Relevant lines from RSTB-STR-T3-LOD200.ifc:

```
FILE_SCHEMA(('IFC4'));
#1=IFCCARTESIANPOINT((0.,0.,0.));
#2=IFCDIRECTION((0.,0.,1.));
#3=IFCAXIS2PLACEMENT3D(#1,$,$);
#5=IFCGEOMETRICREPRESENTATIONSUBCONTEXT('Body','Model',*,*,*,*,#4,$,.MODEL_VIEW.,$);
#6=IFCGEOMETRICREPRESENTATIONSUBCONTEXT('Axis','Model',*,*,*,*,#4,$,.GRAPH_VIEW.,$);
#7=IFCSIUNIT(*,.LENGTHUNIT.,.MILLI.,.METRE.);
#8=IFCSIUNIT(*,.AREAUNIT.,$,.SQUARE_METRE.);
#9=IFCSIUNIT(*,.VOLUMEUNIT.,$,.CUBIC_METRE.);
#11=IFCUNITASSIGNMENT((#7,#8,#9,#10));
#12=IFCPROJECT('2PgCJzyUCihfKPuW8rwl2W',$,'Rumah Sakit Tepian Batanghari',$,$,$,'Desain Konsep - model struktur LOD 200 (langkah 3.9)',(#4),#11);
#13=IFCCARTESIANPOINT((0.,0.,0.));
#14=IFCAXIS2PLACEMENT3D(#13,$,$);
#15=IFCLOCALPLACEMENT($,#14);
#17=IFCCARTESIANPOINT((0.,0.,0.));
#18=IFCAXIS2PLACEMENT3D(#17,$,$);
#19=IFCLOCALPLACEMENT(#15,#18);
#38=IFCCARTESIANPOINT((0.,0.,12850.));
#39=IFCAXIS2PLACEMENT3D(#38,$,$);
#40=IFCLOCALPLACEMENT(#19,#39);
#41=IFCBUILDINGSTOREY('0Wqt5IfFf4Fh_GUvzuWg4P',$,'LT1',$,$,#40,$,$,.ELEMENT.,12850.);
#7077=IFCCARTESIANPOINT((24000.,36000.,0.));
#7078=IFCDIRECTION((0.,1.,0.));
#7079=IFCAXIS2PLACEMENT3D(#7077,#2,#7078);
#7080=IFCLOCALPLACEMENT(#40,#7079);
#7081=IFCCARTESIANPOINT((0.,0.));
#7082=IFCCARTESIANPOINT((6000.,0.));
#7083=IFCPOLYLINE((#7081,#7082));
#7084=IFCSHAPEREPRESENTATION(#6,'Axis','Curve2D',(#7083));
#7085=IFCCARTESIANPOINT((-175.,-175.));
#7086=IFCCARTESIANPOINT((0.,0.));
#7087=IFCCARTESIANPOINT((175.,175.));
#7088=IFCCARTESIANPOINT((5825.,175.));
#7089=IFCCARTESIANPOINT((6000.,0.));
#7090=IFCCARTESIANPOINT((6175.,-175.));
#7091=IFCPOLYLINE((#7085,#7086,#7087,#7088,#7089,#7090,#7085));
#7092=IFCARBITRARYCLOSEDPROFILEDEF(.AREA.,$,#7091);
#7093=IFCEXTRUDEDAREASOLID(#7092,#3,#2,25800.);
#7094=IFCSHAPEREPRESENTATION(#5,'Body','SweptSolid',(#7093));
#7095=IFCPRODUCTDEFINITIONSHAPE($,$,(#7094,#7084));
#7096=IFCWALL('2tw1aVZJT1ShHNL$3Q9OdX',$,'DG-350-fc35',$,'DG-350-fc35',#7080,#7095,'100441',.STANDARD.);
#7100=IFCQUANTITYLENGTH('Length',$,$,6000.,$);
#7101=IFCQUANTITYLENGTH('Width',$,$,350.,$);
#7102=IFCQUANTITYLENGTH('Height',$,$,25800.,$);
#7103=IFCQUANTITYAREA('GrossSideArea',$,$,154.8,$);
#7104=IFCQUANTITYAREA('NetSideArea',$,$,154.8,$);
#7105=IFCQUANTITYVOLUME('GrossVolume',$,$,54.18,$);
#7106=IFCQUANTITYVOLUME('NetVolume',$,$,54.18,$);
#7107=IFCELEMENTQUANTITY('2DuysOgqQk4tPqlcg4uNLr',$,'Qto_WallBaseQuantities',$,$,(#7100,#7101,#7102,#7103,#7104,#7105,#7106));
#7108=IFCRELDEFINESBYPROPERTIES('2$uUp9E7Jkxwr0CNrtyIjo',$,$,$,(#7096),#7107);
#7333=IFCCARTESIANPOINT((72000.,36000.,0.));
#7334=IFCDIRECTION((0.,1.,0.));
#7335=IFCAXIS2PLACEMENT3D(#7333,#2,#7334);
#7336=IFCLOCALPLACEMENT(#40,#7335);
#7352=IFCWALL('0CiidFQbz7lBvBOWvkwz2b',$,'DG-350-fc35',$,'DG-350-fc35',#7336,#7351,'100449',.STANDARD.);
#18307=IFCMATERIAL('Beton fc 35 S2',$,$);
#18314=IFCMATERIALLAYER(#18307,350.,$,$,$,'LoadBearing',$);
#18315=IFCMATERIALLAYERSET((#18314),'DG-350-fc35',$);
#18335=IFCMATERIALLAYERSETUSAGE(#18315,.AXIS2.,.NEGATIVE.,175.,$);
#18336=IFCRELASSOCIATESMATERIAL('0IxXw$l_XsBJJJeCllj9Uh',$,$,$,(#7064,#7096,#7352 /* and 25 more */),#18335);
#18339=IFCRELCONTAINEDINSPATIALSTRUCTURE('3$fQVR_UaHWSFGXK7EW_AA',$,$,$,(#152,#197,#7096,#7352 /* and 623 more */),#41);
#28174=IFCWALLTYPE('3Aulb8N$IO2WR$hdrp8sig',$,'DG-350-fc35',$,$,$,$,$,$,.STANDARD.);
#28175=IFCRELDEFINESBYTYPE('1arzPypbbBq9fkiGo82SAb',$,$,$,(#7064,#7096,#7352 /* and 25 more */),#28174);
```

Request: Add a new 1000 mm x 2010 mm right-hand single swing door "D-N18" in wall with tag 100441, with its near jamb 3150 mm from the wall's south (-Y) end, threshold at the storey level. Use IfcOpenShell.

```python
import numpy as np
import ifcopenshell
import ifcopenshell.api.feature
import ifcopenshell.api.geometry
import ifcopenshell.api.pset
import ifcopenshell.api.root
import ifcopenshell.api.spatial
import ifcopenshell.geom
import ifcopenshell.util.element
import ifcopenshell.util.placement
import ifcopenshell.util.representation
import ifcopenshell.util.shape
import ifcopenshell.util.unit

model = ifcopenshell.open("RSTB-STR-T3-LOD200.ifc")
unit_scale = ifcopenshell.util.unit.calculate_unit_scale(model)
area_scale = ifcopenshell.util.unit.calculate_unit_scale(model, "AREAUNIT")
volume_scale = ifcopenshell.util.unit.calculate_unit_scale(model, "VOLUMEUNIT")
settings = ifcopenshell.geom.settings()


def volume(element):
    """Net volume in cubic metres, openings subtracted."""
    shape = ifcopenshell.geom.create_shape(settings, element)
    return ifcopenshell.util.shape.get_volume(shape.geometry)


wall = model.by_guid("2tw1aVZJT1ShHNL$3Q9OdX")
storey = ifcopenshell.util.element.get_container(wall, ifc_class="IfcBuildingStorey")
context = ifcopenshell.util.representation.get_context(model, "Model", "Body", "MODEL_VIEW")
before = volume(wall)

width, height, from_end, sill = 1, 2.01, 3.15, 0.0  # metres

# The wall runs along its own X axis, and the end named is its -X end.
wall_shape = ifcopenshell.geom.create_shape(settings, wall)
x, y, z = ifcopenshell.util.shape.get_vertices(wall_shape.geometry).T
start = x.min() + from_end
face, thickness = float(y.min()), float(y.max() - y.min())
wall_matrix = ifcopenshell.util.placement.get_local_placement(wall.ObjectPlacement)
level = ifcopenshell.util.placement.get_local_placement(storey.ObjectPlacement)[2, 3]


def in_wall(x, y):
    """Placement at x, y metres in the wall's axes, at sill height."""
    matrix = wall_matrix.copy()
    matrix[:, 3] = wall_matrix @ np.array([x / unit_scale, y / unit_scale, 0.0, 1.0])
    matrix[2, 3] = level + sill / unit_scale
    return matrix


# Opening: a box that overshoots both wall faces by 50 mm.
opening = ifcopenshell.api.root.create_entity(model, ifc_class="IfcOpeningElement", predefined_type="OPENING")
box = ifcopenshell.api.geometry.add_wall_representation(
    model, context=context, length=width, height=height, thickness=thickness + 0.1
)
ifcopenshell.api.geometry.assign_representation(model, product=opening, representation=box)
ifcopenshell.api.geometry.edit_object_placement(model, product=opening, matrix=in_wall(start, face - 0.05), is_si=False)
ifcopenshell.api.feature.add_feature(model, feature=opening, element=wall)

door = ifcopenshell.api.root.create_entity(model, ifc_class="IfcDoor", name="D-N18", predefined_type="DOOR")
door.OverallWidth, door.OverallHeight = width / unit_scale, height / unit_scale
door.OperationType = "SINGLE_SWING_RIGHT"
body = ifcopenshell.api.geometry.add_door_representation(
    model,
    context=context,
    overall_width=door.OverallWidth,
    overall_height=door.OverallHeight,
    operation_type="SINGLE_SWING_RIGHT",
    lining_properties={"LiningDepth": thickness / unit_scale, "ThresholdDepth": thickness / unit_scale},
)
ifcopenshell.api.geometry.assign_representation(model, product=door, representation=body)
ifcopenshell.api.spatial.assign_container(model, products=[door], relating_structure=storey)
ifcopenshell.api.feature.add_filling(model, opening=opening, element=door)

# The lining spans the wall, so the door starts at the wall face.
ifcopenshell.api.geometry.edit_object_placement(model, product=door, matrix=in_wall(start, face), is_si=False)

after = volume(wall)

# Update the wall's stored quantities.
qto = model.by_id(ifcopenshell.util.element.get_pset(wall, "Qto_WallBaseQuantities", should_inherit=False)["id"])
ifcopenshell.api.pset.edit_qto(model, qto=qto, properties={
    "NetSideArea": after / thickness / area_scale,
    "NetVolume": after / volume_scale,
})

print(f"wall volume {before:.3f} -> {after:.3f} m3")

model.write("RSTB-STR-T3-LOD200_edited.ifc")
```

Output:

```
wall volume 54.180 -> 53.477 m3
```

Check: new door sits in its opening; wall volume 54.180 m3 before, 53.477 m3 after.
